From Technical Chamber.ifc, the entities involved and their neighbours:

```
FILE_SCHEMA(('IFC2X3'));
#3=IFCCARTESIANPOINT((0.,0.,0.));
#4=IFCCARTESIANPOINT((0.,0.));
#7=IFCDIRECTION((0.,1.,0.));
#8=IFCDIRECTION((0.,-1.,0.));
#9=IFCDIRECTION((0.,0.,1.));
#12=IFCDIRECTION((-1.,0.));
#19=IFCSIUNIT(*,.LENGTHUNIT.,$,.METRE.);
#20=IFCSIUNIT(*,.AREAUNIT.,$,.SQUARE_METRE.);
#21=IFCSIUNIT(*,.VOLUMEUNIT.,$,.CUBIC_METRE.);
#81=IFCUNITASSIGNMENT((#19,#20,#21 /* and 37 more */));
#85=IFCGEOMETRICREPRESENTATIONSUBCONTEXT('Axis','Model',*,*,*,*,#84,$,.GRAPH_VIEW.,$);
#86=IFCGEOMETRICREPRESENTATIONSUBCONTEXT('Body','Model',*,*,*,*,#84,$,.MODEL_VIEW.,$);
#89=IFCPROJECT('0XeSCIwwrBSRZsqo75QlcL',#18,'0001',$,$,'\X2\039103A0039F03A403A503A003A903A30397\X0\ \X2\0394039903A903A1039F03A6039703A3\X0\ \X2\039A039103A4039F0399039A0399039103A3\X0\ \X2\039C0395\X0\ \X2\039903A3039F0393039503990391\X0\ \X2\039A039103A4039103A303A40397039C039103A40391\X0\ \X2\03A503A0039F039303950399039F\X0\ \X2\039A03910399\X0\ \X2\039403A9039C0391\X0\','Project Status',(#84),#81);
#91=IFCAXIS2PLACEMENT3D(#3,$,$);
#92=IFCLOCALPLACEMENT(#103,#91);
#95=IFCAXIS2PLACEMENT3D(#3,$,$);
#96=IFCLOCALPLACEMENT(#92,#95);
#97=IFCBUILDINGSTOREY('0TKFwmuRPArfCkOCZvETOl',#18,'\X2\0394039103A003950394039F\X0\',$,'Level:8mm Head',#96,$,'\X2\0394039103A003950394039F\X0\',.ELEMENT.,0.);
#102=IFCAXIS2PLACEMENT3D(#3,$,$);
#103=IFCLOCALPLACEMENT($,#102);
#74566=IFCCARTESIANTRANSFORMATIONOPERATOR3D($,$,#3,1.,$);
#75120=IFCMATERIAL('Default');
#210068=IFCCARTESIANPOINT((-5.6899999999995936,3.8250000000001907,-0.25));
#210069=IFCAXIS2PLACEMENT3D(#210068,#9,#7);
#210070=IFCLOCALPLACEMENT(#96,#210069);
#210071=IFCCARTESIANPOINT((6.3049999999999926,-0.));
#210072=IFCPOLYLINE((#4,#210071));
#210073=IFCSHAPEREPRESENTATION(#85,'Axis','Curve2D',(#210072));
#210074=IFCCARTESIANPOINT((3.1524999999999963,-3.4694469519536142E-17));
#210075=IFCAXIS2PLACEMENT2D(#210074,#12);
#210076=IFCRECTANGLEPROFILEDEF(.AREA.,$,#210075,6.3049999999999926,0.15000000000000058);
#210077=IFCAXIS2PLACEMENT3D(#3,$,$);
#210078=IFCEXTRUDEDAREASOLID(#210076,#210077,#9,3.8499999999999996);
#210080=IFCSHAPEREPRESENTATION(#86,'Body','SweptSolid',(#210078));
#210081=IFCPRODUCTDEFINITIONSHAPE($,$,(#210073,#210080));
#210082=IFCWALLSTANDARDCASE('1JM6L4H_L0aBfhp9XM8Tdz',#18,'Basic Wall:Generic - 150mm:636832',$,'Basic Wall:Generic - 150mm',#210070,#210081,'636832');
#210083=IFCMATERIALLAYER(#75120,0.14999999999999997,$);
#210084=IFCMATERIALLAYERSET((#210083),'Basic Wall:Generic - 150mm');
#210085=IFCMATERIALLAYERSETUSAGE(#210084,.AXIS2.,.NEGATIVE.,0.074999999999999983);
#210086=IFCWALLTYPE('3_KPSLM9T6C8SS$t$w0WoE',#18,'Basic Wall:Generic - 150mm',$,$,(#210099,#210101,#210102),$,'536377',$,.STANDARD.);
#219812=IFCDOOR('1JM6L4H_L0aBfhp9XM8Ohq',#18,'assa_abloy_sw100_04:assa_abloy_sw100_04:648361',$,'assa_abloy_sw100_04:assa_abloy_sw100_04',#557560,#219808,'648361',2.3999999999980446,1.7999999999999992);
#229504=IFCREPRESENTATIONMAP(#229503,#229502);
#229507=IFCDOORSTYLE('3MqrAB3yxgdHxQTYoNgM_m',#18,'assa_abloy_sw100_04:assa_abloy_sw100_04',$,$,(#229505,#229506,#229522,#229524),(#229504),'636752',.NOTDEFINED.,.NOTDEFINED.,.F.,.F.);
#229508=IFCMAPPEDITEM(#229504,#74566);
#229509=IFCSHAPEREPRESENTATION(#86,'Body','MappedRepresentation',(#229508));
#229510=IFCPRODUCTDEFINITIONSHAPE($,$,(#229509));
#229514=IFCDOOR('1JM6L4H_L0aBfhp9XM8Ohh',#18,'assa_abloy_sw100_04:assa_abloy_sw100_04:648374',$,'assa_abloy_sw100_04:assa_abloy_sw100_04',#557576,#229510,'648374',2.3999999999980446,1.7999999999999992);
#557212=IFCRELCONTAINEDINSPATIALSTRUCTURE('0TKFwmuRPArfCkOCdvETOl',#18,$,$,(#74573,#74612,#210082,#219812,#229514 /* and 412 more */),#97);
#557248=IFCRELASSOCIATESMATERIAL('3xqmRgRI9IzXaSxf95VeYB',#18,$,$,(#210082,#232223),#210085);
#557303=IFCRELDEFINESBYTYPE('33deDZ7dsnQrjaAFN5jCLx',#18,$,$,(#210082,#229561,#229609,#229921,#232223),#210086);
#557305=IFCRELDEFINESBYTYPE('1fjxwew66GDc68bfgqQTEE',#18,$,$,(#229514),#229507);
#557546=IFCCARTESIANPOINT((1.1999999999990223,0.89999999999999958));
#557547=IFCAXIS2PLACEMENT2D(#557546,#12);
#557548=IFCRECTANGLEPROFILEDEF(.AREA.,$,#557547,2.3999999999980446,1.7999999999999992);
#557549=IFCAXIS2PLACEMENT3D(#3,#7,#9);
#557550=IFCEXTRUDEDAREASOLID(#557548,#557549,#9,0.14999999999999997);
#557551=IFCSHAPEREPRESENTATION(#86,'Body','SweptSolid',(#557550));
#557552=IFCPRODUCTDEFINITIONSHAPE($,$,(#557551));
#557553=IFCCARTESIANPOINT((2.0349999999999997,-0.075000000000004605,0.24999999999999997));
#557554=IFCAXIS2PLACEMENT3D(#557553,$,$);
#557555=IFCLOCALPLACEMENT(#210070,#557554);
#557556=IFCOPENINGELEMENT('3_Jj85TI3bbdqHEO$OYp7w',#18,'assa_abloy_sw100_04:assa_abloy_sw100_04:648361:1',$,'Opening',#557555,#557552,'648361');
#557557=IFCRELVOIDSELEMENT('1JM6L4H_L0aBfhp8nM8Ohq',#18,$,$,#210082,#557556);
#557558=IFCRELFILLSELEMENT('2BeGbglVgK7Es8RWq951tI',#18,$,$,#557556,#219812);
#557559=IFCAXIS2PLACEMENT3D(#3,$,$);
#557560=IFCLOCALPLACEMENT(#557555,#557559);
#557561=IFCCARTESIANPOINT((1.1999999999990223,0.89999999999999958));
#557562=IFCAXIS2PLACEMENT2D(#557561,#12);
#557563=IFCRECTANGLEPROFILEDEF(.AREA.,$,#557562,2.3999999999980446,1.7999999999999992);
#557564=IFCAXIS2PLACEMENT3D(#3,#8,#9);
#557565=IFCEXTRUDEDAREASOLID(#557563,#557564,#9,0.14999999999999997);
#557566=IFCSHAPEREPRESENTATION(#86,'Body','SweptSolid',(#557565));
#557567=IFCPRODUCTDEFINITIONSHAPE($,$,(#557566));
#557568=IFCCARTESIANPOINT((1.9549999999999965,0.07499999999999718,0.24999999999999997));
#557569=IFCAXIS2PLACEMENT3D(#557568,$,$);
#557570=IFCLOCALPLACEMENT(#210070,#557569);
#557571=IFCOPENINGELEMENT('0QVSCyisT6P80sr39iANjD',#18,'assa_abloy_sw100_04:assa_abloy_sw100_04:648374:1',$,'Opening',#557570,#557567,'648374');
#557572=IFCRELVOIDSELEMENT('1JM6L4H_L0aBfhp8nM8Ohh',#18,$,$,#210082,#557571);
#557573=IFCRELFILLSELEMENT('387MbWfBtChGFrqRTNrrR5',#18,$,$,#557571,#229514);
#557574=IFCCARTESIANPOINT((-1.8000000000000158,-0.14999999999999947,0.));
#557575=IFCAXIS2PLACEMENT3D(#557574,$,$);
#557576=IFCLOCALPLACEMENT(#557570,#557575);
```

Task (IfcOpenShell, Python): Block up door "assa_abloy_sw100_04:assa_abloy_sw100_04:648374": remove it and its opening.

```python
import ifcopenshell
import ifcopenshell.api.feature
import ifcopenshell.api.root
import ifcopenshell.geom
import ifcopenshell.util.shape

model = ifcopenshell.open("Technical Chamber.ifc")
settings = ifcopenshell.geom.settings()


def volume(element):
    """Net volume in cubic metres, openings subtracted."""
    shape = ifcopenshell.geom.create_shape(settings, element)
    return ifcopenshell.util.shape.get_volume(shape.geometry)


door = model.by_id(229514)
opening = door.FillsVoids[0].RelatingOpeningElement
wall = opening.VoidsElements[0].RelatingBuildingElement
before = volume(wall)

ifcopenshell.api.root.remove_product(model, product=door)
ifcopenshell.api.feature.remove_feature(model, feature=opening)

after = volume(wall)

print(f"wall volume {before:.3f} -> {after:.3f} m3")

model.write("Technical Chamber_edited.ifc")
```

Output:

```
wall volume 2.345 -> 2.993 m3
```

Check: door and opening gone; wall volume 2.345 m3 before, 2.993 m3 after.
